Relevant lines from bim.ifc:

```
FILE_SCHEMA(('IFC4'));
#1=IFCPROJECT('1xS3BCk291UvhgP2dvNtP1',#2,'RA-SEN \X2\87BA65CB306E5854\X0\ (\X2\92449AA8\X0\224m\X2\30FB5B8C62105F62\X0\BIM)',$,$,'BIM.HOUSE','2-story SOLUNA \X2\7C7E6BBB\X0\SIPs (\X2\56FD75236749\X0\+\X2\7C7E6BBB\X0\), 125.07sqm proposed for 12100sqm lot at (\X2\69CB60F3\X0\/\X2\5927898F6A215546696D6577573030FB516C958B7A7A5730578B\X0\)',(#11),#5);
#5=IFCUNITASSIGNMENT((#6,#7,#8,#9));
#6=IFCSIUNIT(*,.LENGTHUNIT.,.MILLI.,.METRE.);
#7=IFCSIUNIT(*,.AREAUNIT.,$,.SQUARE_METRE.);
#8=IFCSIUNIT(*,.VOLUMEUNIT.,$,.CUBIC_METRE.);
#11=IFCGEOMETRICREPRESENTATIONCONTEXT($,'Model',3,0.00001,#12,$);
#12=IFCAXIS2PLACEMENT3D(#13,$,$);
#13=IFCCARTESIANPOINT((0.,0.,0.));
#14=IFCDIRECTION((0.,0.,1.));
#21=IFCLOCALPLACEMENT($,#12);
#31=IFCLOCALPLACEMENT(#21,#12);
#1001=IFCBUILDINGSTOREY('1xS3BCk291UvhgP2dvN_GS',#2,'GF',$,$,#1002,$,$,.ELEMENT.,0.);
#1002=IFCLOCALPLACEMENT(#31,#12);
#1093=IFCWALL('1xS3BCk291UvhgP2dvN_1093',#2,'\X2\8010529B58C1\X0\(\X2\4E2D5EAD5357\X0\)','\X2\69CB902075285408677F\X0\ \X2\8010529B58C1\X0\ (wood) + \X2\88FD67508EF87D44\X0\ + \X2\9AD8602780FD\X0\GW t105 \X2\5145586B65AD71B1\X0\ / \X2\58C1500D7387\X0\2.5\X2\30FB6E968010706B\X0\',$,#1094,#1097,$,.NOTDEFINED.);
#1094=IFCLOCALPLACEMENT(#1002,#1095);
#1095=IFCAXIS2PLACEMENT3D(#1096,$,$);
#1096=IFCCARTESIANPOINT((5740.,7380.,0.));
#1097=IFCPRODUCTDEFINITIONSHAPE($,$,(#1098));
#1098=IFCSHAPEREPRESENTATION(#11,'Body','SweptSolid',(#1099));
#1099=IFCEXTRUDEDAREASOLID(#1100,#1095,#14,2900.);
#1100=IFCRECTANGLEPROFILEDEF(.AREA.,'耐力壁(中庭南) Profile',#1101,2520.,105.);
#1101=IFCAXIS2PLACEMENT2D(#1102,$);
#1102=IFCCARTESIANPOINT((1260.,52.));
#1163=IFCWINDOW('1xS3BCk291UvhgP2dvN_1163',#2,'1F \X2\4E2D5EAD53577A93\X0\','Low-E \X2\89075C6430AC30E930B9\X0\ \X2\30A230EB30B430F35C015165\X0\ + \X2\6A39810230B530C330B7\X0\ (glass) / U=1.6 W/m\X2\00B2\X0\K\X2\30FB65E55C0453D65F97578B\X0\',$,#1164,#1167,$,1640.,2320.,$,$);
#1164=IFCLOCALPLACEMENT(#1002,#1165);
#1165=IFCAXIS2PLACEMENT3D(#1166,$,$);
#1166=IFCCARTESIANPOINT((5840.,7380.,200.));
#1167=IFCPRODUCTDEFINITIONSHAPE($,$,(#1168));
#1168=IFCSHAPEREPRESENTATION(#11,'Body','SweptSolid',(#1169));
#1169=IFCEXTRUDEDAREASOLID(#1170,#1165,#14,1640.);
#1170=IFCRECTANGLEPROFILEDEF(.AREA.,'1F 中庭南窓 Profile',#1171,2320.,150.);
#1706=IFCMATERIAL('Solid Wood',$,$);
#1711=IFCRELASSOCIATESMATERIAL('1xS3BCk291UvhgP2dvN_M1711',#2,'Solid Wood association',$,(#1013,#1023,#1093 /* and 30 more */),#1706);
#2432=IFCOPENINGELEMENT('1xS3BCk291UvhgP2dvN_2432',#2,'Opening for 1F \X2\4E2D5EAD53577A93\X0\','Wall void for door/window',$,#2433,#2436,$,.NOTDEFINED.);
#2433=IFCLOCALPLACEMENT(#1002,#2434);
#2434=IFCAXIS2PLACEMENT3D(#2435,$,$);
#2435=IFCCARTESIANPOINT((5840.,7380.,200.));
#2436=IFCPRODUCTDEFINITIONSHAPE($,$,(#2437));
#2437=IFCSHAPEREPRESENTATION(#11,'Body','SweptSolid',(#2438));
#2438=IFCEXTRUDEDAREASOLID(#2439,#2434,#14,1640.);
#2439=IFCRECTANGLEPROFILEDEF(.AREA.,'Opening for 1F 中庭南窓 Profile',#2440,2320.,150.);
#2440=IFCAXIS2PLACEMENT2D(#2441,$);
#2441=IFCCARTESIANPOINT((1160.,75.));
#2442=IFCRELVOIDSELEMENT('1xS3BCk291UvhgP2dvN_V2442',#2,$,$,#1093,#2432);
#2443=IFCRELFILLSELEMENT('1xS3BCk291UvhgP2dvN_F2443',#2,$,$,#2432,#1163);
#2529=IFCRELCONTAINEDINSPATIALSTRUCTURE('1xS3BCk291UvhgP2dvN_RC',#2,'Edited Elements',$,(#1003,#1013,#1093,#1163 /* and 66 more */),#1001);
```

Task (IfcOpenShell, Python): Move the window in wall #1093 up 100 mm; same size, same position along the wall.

```python
import numpy as np
import ifcopenshell
import ifcopenshell.api.geometry
import ifcopenshell.util.placement
import ifcopenshell.util.unit

model = ifcopenshell.open("bim.ifc")
unit_scale = ifcopenshell.util.unit.calculate_unit_scale(model)

window = model.by_id(1163)
opening = window.FillsVoids[0].RelatingOpeningElement
dz = 100.0

shift = np.array([0.0, 0.0, dz])
# The window is not placed relative to its opening, so move both.
for product in (opening, window):
    matrix = ifcopenshell.util.placement.get_local_placement(product.ObjectPlacement)
    matrix[:3, 3] += shift
    ifcopenshell.api.geometry.edit_object_placement(model, product=product, matrix=matrix, is_si=False)

print(f"moved by {dz * unit_scale:+.3f} m")

model.write("bim_v2.ifc")
```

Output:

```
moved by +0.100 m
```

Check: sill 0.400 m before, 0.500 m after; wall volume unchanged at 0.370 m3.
